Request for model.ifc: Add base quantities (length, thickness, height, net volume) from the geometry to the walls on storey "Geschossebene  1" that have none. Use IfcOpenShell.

First a look at what the model holds.

```python
import ifcopenshell
import ifcopenshell.util.element
import ifcopenshell.util.unit

model = ifcopenshell.open("model.ifc")
print(model.schema)
for unit_type in ("LENGTHUNIT", "AREAUNIT", "VOLUMEUNIT"):
    print(unit_type, ifcopenshell.util.unit.calculate_unit_scale(model, unit_type))
storey = next(s for s in model.by_type("IfcBuildingStorey") if s.Name == "Geschossebene  1")
walls = [e for e in ifcopenshell.util.element.get_decomposition(storey) if e.is_a("IfcWall")]
for e in sorted(walls, key=lambda e: e.id()):
    print(e.id(), e.is_a(), e.Name, list(ifcopenshell.util.element.get_psets(e, qtos_only=True)), sep=" | ")
```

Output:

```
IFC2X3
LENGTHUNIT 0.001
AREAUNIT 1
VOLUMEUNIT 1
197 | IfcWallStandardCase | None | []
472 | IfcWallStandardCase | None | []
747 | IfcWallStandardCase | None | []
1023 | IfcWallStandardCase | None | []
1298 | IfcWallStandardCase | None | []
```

```python
import ifcopenshell
import ifcopenshell.api.pset
import ifcopenshell.geom
import ifcopenshell.util.element
import ifcopenshell.util.shape
import ifcopenshell.util.unit

model = ifcopenshell.open("model.ifc")
unit_scale = ifcopenshell.util.unit.calculate_unit_scale(model)
volume_scale = ifcopenshell.util.unit.calculate_unit_scale(model, "VOLUMEUNIT")
settings = ifcopenshell.geom.settings()

storey = next(s for s in model.by_type("IfcBuildingStorey") if s.Name == "Geschossebene  1")
walls = [e for e in ifcopenshell.util.element.get_decomposition(storey) if e.is_a("IfcWall")]

for e in sorted(walls, key=lambda e: e.id()):
    if ifcopenshell.util.element.get_psets(e, qtos_only=True, should_inherit=False):
        continue
    # Geometry comes back in metres, in the element's own axes.
    shape = ifcopenshell.geom.create_shape(settings, e)
    values = {
        "Length": ifcopenshell.util.shape.get_x(shape.geometry) / unit_scale,
        "Width": ifcopenshell.util.shape.get_y(shape.geometry) / unit_scale,
        "Height": ifcopenshell.util.shape.get_z(shape.geometry) / unit_scale,
        "NetVolume": ifcopenshell.util.shape.get_volume(shape.geometry) / volume_scale,
    }
    qto = ifcopenshell.api.pset.add_qto(model, product=e, name="BaseQuantities")
    ifcopenshell.api.pset.edit_qto(model, qto=qto, properties=values)
    print(e.id(), {k: round(v, 3) for k, v in values.items()})

model.write("model_rev.ifc")
```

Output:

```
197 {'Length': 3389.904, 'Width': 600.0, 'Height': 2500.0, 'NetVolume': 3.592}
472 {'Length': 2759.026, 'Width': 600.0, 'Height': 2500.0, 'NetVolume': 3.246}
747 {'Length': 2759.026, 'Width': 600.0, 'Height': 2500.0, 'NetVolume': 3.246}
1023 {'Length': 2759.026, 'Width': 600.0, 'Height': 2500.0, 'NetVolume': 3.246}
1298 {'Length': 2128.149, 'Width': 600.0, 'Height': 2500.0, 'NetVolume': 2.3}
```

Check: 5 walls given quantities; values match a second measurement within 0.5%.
